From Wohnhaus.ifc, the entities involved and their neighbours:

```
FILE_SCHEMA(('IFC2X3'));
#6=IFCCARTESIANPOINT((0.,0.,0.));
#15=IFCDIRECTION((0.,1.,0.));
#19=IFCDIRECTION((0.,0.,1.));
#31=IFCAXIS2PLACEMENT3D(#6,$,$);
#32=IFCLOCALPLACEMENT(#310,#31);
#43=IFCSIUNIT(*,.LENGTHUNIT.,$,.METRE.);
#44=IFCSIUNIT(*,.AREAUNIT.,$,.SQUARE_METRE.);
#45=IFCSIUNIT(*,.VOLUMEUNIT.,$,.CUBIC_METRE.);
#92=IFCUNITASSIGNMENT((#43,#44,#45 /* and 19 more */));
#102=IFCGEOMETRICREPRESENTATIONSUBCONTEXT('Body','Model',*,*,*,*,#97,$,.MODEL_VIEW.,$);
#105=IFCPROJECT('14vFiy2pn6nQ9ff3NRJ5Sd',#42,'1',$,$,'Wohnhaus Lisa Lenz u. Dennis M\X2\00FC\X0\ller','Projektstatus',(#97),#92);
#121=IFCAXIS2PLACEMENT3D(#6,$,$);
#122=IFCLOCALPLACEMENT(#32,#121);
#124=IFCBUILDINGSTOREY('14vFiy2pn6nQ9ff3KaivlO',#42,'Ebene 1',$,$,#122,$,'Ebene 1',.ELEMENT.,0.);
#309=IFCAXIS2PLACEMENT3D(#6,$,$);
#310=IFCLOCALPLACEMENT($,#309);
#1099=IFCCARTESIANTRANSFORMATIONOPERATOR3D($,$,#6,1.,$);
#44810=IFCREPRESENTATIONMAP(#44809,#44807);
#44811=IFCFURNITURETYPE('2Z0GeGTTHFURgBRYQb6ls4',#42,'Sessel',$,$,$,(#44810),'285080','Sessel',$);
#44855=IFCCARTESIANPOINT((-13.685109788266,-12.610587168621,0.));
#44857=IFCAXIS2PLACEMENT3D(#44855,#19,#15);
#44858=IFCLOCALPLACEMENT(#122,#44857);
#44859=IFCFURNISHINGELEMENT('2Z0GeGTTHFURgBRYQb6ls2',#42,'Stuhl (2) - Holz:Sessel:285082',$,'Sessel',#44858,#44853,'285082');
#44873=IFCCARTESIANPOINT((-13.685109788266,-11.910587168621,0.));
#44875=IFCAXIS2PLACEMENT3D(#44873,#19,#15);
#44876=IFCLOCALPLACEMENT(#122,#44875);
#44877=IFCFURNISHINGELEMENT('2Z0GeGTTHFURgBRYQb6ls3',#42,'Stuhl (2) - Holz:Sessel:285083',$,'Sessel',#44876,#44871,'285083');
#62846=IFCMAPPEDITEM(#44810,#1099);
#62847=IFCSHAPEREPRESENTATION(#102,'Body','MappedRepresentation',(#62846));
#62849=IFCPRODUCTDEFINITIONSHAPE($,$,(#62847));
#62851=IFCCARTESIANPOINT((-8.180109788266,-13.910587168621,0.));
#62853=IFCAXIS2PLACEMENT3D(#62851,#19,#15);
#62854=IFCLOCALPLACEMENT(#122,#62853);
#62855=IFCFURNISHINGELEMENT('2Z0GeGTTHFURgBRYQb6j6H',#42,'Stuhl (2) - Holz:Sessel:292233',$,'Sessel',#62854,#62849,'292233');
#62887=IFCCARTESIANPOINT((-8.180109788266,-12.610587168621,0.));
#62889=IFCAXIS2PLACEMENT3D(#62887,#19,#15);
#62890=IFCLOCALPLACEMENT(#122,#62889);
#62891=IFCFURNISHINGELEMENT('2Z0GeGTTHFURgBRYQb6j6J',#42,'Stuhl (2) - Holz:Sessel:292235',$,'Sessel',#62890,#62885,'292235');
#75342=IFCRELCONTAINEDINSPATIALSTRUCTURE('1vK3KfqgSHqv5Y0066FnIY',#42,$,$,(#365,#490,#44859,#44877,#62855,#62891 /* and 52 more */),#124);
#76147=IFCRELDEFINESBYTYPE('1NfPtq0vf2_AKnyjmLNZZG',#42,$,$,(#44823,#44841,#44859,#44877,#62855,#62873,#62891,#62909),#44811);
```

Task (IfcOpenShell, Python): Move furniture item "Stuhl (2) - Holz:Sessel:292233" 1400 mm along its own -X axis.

```python
import ifcopenshell
import ifcopenshell.api.geometry
import ifcopenshell.util.placement
import ifcopenshell.util.unit

model = ifcopenshell.open("Wohnhaus.ifc")
unit_scale = ifcopenshell.util.unit.calculate_unit_scale(model)

item = model.by_guid("2Z0GeGTTHFURgBRYQb6j6H")
matrix = ifcopenshell.util.placement.get_local_placement(item.ObjectPlacement)
matrix[:3, 3] -= matrix[:3, 0] * 1.4 / unit_scale
ifcopenshell.api.geometry.edit_object_placement(model, product=item, matrix=matrix, is_si=False)

print(ifcopenshell.util.placement.get_local_placement(item.ObjectPlacement).round(3) + 0.0)

model.write("Wohnhaus-out.ifc")
```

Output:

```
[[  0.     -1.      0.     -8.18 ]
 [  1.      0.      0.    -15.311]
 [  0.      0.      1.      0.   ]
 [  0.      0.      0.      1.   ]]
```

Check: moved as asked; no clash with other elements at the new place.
